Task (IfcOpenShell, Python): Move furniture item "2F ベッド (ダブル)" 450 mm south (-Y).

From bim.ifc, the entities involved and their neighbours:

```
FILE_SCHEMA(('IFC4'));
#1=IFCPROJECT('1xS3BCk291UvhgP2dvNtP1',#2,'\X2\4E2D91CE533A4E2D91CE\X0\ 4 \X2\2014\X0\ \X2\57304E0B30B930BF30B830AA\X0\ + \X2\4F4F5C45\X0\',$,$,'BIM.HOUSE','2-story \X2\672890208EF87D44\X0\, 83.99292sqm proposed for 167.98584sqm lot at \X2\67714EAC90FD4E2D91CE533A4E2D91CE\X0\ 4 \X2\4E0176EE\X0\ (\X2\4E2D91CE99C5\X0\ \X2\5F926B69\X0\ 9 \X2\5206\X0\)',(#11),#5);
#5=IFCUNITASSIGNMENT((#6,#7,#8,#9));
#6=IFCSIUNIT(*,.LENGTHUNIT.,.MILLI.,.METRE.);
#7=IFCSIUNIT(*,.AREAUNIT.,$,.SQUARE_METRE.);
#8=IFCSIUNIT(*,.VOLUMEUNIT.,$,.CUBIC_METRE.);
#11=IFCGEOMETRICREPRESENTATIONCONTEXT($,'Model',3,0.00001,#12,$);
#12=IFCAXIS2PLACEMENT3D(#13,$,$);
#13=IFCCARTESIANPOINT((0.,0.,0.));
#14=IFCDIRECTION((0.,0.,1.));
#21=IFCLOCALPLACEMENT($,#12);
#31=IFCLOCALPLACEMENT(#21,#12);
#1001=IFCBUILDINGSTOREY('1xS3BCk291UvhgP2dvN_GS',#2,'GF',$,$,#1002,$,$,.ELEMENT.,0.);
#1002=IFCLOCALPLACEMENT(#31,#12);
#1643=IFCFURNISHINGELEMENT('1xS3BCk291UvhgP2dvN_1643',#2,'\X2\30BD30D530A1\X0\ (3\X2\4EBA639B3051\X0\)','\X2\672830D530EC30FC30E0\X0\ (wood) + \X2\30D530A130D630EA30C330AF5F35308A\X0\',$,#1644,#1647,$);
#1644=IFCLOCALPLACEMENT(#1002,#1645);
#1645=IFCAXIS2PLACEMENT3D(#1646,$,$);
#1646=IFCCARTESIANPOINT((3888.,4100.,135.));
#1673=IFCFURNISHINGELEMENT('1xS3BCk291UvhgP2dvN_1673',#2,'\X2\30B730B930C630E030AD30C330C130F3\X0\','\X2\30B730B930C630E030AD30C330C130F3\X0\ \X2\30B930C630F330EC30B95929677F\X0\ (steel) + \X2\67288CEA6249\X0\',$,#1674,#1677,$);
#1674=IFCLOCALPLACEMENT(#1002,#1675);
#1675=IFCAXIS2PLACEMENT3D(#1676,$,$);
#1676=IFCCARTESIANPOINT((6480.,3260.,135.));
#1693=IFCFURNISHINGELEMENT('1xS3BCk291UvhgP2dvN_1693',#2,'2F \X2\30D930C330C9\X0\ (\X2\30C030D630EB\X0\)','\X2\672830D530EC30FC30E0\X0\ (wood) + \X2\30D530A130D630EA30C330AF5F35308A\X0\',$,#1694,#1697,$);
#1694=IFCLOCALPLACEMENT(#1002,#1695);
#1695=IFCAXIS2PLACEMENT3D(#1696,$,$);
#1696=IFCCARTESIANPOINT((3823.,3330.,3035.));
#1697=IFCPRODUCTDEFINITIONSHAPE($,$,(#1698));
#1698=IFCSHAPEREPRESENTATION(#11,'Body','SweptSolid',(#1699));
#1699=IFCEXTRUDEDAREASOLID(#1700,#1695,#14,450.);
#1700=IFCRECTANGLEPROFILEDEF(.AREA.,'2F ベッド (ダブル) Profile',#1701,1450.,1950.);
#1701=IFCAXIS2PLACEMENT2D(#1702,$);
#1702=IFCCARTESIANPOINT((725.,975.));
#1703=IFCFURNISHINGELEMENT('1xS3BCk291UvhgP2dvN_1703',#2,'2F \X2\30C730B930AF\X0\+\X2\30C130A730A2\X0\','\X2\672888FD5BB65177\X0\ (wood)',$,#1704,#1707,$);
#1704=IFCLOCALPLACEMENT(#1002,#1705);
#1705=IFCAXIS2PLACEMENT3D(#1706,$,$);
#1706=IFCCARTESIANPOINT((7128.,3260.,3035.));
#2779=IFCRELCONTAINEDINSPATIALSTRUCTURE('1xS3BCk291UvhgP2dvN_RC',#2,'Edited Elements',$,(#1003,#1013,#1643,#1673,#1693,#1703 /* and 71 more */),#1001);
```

```python
import ifcopenshell
import ifcopenshell.api.geometry
import ifcopenshell.util.placement
import ifcopenshell.util.unit

model = ifcopenshell.open("bim.ifc")
unit_scale = ifcopenshell.util.unit.calculate_unit_scale(model)

item = model.by_id(1693)
matrix = ifcopenshell.util.placement.get_local_placement(item.ObjectPlacement)
matrix[1, 3] -= 0.45 / unit_scale
ifcopenshell.api.geometry.edit_object_placement(model, product=item, matrix=matrix, is_si=False)

print(ifcopenshell.util.placement.get_local_placement(item.ObjectPlacement).round(3) + 0.0)

model.write("bim-out.ifc")
```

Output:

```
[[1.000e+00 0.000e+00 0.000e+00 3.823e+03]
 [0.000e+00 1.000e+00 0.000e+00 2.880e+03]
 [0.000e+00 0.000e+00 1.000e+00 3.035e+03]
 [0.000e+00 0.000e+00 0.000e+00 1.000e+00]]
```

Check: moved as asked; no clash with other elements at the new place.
